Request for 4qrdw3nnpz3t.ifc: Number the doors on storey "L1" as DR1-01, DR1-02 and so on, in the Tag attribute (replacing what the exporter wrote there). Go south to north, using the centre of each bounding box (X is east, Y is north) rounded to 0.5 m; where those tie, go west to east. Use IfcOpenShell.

First a look at what the model holds.

```python
import ifcopenshell
import ifcopenshell.util.element
import ifcopenshell.util.placement

model = ifcopenshell.open("4qrdw3nnpz3t.ifc")
print(model.schema)
storey = next(s for s in model.by_type("IfcBuildingStorey") if s.Name == "L1")
doors = [e for e in ifcopenshell.util.element.get_decomposition(storey) if e.is_a("IfcDoor")]
for e in sorted(doors, key=lambda e: e.id()):
    origin = ifcopenshell.util.placement.get_local_placement(e.ObjectPlacement)[:3, 3]
    print(e.id(), e.Tag, e.Name, origin.round(2) + 0.0, sep=" | ")
```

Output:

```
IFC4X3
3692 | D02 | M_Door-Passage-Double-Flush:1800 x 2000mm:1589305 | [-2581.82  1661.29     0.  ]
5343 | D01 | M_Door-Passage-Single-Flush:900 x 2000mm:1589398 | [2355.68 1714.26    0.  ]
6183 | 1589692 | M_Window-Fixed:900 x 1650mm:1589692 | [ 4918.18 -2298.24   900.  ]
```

```python
import ifcopenshell
import ifcopenshell.geom
import ifcopenshell.util.element
import ifcopenshell.util.shape

model = ifcopenshell.open("4qrdw3nnpz3t.ifc")
settings = ifcopenshell.geom.settings()
settings.set("use-world-coords", True)


def centre(element):
    shape = ifcopenshell.geom.create_shape(settings, element)
    return ifcopenshell.util.shape.get_bbox_centroid(shape.geometry)


storey = next(s for s in model.by_type("IfcBuildingStorey") if s.Name == "L1")
doors = [e for e in ifcopenshell.util.element.get_decomposition(storey) if e.is_a("IfcDoor")]

# Insertion points can sit at a corner or the storey origin, so sort by the geometry (in metres).
centres = {e: centre(e) for e in doors}
doors.sort(key=lambda e: (round(centres[e][1] / 0.5), centres[e][0]))

for i, e in enumerate(doors, start=1):
    number = f"DR1-{i:02d}"
    e.Tag = number
    print(e.id(), number)

model.write("4qrdw3nnpz3t_updated.ifc")
```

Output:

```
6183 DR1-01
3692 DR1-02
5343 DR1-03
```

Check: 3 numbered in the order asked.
